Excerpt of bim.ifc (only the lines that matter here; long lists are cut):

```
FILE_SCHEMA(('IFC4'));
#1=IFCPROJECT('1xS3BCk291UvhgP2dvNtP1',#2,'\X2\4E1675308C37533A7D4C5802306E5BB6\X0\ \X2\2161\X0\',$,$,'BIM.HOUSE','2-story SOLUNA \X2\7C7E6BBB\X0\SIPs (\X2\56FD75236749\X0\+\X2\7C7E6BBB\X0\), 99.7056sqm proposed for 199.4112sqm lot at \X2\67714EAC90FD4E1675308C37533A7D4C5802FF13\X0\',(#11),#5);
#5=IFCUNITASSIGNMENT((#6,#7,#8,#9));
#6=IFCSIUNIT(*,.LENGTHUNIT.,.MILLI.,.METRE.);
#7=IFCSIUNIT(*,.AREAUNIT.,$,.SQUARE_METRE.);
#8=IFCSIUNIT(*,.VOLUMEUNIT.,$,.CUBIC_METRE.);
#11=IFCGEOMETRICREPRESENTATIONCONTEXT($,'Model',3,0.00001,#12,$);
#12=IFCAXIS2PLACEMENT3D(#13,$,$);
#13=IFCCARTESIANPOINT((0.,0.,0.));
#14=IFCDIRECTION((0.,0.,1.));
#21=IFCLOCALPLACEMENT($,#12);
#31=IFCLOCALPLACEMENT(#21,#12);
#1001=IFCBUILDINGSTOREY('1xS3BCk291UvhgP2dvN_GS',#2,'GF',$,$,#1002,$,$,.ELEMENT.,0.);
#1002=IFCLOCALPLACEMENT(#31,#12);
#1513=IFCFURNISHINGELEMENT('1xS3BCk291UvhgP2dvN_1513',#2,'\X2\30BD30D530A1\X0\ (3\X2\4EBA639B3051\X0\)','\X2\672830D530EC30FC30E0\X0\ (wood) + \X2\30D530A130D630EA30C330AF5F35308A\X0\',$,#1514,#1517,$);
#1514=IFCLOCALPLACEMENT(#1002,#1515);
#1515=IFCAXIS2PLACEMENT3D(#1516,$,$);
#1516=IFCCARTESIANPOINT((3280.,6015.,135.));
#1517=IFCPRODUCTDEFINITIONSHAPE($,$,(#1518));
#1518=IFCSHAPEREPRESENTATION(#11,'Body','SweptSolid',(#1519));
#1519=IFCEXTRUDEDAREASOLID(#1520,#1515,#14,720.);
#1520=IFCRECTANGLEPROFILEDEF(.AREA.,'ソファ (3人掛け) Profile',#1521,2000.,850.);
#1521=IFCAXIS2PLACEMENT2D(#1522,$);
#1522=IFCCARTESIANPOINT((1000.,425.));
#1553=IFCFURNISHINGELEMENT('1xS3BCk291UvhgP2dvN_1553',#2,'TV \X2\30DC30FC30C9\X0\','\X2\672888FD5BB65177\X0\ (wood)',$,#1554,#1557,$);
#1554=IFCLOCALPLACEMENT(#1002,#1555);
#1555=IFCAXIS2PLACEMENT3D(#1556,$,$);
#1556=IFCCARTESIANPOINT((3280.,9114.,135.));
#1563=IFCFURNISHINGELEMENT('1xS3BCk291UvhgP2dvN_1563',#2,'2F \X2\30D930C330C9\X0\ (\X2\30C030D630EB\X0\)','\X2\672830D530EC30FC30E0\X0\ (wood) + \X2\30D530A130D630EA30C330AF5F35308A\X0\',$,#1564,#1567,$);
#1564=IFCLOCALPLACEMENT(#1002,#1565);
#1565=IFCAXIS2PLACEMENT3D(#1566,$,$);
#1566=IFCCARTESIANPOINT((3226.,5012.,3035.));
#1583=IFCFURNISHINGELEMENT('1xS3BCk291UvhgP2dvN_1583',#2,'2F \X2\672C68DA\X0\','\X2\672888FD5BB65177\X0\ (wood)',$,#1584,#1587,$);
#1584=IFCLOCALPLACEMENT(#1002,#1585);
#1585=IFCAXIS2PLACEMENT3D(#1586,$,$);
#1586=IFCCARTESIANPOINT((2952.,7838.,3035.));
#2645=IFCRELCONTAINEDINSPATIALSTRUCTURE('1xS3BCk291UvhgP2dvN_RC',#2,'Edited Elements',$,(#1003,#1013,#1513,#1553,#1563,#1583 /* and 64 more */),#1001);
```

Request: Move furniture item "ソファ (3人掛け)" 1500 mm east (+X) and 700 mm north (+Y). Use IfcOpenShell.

```python
import ifcopenshell
import ifcopenshell.api.geometry
import ifcopenshell.util.placement
import ifcopenshell.util.unit

model = ifcopenshell.open("bim.ifc")
unit_scale = ifcopenshell.util.unit.calculate_unit_scale(model)

item = model.by_guid("1xS3BCk291UvhgP2dvN_1513")
matrix = ifcopenshell.util.placement.get_local_placement(item.ObjectPlacement)
matrix[0, 3] += 1.5 / unit_scale
matrix[1, 3] += 0.7 / unit_scale
ifcopenshell.api.geometry.edit_object_placement(model, product=item, matrix=matrix, is_si=False)

print(ifcopenshell.util.placement.get_local_placement(item.ObjectPlacement).round(3) + 0.0)

model.write("bim_updated.ifc")
```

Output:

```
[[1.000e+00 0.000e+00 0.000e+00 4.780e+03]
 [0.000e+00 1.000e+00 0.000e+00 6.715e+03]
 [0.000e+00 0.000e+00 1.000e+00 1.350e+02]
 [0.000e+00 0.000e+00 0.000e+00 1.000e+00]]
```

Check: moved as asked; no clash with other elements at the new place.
